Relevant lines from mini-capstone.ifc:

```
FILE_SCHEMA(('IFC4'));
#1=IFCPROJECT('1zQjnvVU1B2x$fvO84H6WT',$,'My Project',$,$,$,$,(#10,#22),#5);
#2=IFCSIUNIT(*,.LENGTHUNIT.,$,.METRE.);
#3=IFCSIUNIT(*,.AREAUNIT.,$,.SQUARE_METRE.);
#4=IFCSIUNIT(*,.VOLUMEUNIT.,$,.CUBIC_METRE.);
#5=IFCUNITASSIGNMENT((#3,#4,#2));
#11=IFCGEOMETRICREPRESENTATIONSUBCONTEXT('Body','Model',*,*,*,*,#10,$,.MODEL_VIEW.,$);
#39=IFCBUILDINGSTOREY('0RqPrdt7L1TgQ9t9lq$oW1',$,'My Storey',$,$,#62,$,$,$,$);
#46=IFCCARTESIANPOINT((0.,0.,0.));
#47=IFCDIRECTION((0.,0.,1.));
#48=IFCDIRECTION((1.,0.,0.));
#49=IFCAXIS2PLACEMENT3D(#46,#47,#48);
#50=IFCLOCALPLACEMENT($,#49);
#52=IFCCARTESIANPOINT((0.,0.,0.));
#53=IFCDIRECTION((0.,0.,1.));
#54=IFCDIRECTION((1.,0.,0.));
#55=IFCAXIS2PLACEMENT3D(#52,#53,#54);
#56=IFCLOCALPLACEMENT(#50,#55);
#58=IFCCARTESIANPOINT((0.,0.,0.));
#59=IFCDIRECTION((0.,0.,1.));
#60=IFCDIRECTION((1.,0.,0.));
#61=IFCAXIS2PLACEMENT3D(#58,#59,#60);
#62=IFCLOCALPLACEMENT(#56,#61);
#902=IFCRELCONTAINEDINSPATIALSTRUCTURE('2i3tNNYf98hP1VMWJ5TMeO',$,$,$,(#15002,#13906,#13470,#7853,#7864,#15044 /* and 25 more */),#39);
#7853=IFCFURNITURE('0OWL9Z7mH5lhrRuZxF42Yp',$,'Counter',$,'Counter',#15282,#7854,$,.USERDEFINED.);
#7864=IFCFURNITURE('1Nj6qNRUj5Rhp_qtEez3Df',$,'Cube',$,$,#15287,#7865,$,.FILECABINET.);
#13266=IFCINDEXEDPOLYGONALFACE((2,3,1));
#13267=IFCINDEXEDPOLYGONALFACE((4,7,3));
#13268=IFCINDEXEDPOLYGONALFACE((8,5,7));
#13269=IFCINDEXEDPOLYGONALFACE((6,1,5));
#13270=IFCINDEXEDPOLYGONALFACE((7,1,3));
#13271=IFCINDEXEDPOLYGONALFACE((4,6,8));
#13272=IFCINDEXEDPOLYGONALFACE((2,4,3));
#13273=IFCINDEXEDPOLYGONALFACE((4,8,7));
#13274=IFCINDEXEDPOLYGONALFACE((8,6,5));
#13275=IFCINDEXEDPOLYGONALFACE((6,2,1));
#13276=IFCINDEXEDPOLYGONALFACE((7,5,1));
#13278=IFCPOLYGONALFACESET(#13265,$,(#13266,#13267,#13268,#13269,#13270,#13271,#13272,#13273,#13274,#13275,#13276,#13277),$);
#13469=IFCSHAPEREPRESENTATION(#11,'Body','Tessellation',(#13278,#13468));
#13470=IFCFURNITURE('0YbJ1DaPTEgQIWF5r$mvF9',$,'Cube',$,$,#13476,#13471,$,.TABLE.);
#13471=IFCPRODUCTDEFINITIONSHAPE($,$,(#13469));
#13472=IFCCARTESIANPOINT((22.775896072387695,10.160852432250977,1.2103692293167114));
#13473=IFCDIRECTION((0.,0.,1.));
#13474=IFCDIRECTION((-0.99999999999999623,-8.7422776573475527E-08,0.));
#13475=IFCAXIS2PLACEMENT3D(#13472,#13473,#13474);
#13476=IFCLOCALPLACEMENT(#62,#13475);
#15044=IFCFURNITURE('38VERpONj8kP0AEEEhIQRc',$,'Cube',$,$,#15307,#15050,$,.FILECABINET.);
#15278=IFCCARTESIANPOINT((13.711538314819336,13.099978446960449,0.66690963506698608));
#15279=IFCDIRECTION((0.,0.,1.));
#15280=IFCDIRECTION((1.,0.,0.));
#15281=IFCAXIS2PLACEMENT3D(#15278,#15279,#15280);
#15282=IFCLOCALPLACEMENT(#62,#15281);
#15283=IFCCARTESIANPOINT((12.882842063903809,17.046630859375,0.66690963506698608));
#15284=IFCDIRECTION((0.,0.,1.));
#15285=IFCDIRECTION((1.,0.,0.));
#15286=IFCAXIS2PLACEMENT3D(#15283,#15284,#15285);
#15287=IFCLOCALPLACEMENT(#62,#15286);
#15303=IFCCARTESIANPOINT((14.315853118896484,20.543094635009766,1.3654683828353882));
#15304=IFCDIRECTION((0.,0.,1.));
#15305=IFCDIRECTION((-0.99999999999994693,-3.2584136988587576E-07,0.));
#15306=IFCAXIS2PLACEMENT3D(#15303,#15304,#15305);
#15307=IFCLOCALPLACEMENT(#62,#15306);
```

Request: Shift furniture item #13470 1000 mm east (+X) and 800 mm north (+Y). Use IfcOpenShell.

```python
import ifcopenshell
import ifcopenshell.api.geometry
import ifcopenshell.util.placement
import ifcopenshell.util.unit

model = ifcopenshell.open("mini-capstone.ifc")
unit_scale = ifcopenshell.util.unit.calculate_unit_scale(model)

item = model.by_id(13470)
matrix = ifcopenshell.util.placement.get_local_placement(item.ObjectPlacement)
matrix[0, 3] += 1 / unit_scale
matrix[1, 3] += 0.8 / unit_scale
ifcopenshell.api.geometry.edit_object_placement(model, product=item, matrix=matrix, is_si=False)

print(ifcopenshell.util.placement.get_local_placement(item.ObjectPlacement).round(3) + 0.0)

model.write("mini-capstone_rev.ifc")
```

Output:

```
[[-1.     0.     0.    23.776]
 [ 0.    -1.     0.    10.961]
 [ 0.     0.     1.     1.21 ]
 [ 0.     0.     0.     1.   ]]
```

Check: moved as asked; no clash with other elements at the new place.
